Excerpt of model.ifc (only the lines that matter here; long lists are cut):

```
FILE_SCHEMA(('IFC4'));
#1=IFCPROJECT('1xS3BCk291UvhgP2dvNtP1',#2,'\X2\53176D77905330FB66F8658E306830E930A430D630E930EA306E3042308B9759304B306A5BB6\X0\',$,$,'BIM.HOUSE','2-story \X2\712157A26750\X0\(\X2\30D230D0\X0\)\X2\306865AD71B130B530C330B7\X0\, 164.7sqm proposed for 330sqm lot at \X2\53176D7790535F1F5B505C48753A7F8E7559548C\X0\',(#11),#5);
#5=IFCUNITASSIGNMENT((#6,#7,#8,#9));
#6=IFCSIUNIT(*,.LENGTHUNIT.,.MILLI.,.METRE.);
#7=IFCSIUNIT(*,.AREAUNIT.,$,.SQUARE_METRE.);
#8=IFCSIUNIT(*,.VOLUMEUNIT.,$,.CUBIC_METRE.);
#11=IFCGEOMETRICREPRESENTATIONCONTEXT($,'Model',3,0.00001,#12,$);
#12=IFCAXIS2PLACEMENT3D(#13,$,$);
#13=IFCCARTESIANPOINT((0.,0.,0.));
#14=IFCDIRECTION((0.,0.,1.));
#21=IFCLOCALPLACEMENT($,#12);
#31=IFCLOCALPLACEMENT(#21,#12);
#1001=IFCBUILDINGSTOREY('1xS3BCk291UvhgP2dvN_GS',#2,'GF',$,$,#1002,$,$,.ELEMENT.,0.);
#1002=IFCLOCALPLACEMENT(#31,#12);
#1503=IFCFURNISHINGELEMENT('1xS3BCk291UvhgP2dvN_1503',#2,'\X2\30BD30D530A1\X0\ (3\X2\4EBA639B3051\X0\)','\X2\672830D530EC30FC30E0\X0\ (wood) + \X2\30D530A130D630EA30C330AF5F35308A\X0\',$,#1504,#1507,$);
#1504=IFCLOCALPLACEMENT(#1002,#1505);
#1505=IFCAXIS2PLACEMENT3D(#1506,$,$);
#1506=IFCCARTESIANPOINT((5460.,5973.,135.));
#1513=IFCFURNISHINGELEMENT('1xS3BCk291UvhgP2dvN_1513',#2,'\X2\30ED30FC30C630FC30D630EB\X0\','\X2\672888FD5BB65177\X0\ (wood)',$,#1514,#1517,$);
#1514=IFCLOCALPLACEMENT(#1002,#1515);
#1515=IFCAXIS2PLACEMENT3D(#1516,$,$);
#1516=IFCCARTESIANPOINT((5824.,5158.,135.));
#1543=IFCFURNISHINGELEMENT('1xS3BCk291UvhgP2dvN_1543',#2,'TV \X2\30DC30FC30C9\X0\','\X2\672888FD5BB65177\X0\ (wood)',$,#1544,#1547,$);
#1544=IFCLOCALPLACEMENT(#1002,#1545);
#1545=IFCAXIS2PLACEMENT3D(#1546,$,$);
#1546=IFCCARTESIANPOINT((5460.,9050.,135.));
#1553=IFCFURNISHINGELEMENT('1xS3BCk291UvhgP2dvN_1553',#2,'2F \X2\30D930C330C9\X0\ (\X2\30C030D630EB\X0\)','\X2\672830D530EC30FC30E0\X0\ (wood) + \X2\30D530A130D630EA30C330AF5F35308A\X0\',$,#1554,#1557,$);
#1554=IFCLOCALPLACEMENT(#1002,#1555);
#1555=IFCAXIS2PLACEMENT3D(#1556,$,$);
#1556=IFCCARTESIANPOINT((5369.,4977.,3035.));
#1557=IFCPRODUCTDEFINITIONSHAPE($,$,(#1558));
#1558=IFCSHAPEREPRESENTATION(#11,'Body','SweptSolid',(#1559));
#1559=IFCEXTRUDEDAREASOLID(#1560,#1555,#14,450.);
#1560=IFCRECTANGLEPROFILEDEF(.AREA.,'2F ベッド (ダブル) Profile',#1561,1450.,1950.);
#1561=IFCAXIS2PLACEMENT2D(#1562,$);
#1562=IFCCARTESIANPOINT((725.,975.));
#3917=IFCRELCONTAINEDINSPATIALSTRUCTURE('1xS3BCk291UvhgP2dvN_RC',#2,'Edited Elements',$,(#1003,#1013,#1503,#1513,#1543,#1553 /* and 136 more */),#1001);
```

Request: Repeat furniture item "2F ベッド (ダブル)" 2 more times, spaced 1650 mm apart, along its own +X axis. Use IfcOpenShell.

```python
import ifcopenshell
import ifcopenshell.api.geometry
import ifcopenshell.api.root
import ifcopenshell.util.element
import ifcopenshell.util.placement

model = ifcopenshell.open("model.ifc")


def reuse_history(source, copy):
    """copy_class also copies each property set's owner history, people and application; keep the originals."""
    for rel in copy.IsDefinedBy:
        if rel.is_a("IfcRelDefinesByProperties") and (history := rel.RelatingPropertyDefinition.OwnerHistory):
            rel.RelatingPropertyDefinition.OwnerHistory = source.OwnerHistory
            ifcopenshell.util.element.remove_deep2(model, history)


source = model.by_id(1553)
base = ifcopenshell.util.placement.get_local_placement(source.ObjectPlacement)
step = base[:3, 0] * 1650.0

for i in range(1, 3):
    copy = ifcopenshell.api.root.copy_class(model, product=source)
    copy.Representation = ifcopenshell.util.element.copy_deep(
        model, source.Representation, exclude=["IfcGeometricRepresentationContext", "IfcRepresentationMap"]
    )
    reuse_history(source, copy)
    matrix = base.copy()
    matrix[:3, 3] += i * step
    print("added at", matrix[:3, 3].round(3) + 0.0)
    ifcopenshell.api.geometry.edit_object_placement(model, product=copy, matrix=matrix, is_si=False)

model.write("model_updated.ifc")
```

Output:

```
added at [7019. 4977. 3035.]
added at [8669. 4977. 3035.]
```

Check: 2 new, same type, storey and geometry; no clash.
